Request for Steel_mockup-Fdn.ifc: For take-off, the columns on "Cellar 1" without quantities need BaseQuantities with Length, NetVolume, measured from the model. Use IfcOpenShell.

First a look at what the model holds.

```python
import ifcopenshell
import ifcopenshell.util.element
import ifcopenshell.util.unit

model = ifcopenshell.open("Steel_mockup-Fdn.ifc")
print(model.schema)
for unit_type in ("LENGTHUNIT", "AREAUNIT", "VOLUMEUNIT"):
    print(unit_type, ifcopenshell.util.unit.calculate_unit_scale(model, unit_type))
storey = next(s for s in model.by_type("IfcBuildingStorey") if s.Name == "Cellar 1")
columns = [e for e in ifcopenshell.util.element.get_decomposition(storey) if e.is_a("IfcColumn")]
for e in sorted(columns, key=lambda e: e.id()):
    print(e.id(), e.is_a(), e.Name, list(ifcopenshell.util.element.get_psets(e, qtos_only=True)), sep=" | ")
```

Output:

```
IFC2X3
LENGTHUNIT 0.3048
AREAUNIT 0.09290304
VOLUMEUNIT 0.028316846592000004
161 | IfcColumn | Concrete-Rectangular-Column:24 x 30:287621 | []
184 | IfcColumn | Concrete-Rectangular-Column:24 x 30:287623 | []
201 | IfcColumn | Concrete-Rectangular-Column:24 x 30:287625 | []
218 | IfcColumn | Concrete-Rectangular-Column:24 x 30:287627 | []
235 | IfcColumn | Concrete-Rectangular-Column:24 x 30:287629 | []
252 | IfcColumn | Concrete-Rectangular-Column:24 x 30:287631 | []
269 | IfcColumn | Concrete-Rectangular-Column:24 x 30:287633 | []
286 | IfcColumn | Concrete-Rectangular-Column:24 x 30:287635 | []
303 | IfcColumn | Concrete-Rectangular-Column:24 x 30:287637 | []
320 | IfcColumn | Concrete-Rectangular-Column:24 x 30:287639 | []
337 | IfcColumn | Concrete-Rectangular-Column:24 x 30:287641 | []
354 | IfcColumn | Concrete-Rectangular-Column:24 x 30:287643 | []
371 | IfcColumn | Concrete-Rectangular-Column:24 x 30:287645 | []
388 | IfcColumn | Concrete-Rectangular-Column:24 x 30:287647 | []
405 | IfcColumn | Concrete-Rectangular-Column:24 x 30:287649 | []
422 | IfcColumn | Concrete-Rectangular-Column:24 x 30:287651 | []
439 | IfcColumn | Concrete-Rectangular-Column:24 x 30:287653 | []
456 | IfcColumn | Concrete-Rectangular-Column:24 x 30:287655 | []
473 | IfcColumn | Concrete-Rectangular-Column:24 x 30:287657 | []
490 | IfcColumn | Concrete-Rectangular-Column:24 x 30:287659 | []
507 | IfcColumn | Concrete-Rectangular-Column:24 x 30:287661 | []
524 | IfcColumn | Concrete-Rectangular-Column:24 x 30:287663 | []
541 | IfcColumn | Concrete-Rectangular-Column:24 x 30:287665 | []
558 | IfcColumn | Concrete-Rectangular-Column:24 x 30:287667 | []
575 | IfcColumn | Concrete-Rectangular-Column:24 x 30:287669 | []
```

```python
import ifcopenshell
import ifcopenshell.api.pset
import ifcopenshell.geom
import ifcopenshell.util.element
import ifcopenshell.util.shape
import ifcopenshell.util.unit

model = ifcopenshell.open("Steel_mockup-Fdn.ifc")
unit_scale = ifcopenshell.util.unit.calculate_unit_scale(model)
volume_scale = ifcopenshell.util.unit.calculate_unit_scale(model, "VOLUMEUNIT")
settings = ifcopenshell.geom.settings()

storey = next(s for s in model.by_type("IfcBuildingStorey") if s.Name == "Cellar 1")
columns = [e for e in ifcopenshell.util.element.get_decomposition(storey) if e.is_a("IfcColumn")]

for e in sorted(columns, key=lambda e: e.id()):
    if ifcopenshell.util.element.get_psets(e, qtos_only=True, should_inherit=False):
        continue
    # Geometry comes back in metres, in the element's own axes.
    shape = ifcopenshell.geom.create_shape(settings, e)
    values = {
        "Length": ifcopenshell.util.shape.get_z(shape.geometry) / unit_scale,
        "NetVolume": ifcopenshell.util.shape.get_volume(shape.geometry) / volume_scale,
    }
    qto = ifcopenshell.api.pset.add_qto(model, product=e, name="BaseQuantities")
    ifcopenshell.api.pset.edit_qto(model, qto=qto, properties=values)
    print(e.id(), {k: round(v, 3) for k, v in values.items()})

model.write("Steel_mockup-Fdn_updated.ifc")
```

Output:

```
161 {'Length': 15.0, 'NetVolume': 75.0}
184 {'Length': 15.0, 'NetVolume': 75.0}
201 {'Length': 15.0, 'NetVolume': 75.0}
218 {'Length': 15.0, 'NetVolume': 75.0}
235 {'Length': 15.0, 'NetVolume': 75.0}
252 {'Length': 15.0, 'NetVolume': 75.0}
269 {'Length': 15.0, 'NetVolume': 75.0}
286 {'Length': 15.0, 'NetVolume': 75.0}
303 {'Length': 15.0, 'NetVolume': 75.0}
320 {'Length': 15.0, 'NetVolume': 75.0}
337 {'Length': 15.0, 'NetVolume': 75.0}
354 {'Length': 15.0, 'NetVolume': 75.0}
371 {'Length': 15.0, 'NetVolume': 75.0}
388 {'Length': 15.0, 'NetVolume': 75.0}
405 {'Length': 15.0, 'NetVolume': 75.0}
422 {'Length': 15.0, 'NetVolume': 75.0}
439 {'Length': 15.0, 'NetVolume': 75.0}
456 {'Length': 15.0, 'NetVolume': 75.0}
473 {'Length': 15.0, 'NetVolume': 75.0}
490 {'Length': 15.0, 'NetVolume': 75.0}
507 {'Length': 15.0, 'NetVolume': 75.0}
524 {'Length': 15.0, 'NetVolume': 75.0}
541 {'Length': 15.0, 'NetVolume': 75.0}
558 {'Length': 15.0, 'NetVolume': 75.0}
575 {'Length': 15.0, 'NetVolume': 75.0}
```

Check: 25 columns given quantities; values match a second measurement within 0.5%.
